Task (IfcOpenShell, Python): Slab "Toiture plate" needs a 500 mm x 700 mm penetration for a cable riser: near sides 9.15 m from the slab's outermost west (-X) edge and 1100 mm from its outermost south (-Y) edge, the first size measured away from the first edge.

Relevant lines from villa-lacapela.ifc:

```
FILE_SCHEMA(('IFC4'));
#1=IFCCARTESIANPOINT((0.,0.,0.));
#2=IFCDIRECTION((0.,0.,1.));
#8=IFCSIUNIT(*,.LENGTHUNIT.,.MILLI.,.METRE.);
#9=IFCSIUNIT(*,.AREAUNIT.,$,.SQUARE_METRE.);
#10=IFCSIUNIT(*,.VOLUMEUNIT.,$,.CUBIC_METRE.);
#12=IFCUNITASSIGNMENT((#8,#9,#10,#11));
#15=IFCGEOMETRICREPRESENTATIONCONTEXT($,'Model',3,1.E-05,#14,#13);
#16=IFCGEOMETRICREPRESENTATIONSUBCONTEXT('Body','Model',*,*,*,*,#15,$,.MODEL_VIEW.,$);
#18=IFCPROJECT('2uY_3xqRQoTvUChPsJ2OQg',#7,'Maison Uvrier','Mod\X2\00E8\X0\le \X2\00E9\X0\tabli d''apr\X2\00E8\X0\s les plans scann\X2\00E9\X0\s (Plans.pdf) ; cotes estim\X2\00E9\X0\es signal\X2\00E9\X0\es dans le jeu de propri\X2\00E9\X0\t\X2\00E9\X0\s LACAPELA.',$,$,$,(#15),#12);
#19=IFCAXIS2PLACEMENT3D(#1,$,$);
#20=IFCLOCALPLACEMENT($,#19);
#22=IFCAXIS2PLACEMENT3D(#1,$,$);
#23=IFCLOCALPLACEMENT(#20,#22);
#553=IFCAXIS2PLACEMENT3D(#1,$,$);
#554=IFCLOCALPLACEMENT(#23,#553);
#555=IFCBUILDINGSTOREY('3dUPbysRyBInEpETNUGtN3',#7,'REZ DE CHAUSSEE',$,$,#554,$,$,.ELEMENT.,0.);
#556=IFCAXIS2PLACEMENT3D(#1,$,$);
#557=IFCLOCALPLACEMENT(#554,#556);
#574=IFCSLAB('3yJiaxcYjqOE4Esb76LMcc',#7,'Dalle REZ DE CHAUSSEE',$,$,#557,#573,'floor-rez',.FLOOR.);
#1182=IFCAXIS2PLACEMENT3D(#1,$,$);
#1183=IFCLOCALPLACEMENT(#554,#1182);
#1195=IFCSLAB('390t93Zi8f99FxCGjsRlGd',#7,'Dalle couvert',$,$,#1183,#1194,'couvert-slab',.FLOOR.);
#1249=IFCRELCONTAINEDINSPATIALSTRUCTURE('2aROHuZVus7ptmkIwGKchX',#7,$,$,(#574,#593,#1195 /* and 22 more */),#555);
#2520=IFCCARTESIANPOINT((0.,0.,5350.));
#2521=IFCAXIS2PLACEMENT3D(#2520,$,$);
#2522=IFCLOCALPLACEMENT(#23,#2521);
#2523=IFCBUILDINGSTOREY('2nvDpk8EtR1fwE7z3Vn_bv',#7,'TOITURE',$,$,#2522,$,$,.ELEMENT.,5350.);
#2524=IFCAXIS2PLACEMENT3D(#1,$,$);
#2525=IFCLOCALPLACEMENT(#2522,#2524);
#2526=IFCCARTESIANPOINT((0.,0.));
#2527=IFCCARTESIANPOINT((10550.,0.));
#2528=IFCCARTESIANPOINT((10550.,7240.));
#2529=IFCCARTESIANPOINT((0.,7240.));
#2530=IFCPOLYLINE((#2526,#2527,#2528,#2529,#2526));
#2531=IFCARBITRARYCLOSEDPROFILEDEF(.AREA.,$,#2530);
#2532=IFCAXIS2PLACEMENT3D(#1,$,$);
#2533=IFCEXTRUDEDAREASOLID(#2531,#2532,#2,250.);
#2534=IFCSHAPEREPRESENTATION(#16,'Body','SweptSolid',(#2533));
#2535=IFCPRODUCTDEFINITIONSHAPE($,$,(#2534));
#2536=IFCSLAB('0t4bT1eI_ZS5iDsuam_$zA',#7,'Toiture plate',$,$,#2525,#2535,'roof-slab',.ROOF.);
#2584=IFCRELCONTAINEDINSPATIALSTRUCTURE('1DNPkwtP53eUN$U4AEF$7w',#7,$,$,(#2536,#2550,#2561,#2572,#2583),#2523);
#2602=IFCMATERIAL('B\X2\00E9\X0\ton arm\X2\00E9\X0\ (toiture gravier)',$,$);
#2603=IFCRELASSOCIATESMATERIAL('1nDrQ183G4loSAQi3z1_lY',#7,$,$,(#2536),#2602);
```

```python
import numpy as np
import ifcopenshell
import ifcopenshell.api.feature
import ifcopenshell.api.geometry
import ifcopenshell.api.root
import ifcopenshell.geom
import ifcopenshell.util.placement
import ifcopenshell.util.representation
import ifcopenshell.util.shape
import ifcopenshell.util.unit

model = ifcopenshell.open("villa-lacapela.ifc")
unit_scale = ifcopenshell.util.unit.calculate_unit_scale(model)
settings = ifcopenshell.geom.settings()


def volume(element):
    """Net volume in cubic metres, openings subtracted."""
    shape = ifcopenshell.geom.create_shape(settings, element)
    return ifcopenshell.util.shape.get_volume(shape.geometry)


slab = model.by_guid("0t4bT1eI_ZS5iDsuam_$zA")
before = volume(slab)

# Extent in the slab's own axes, in metres. The edges named are its -X and -Y sides.
slab_shape = ifcopenshell.geom.create_shape(settings, slab)
vertices = ifcopenshell.util.shape.get_vertices(slab_shape.geometry)
x_min, y_min, bottom = vertices.min(axis=0)
top = vertices[:, 2].max()

opening = ifcopenshell.api.root.create_entity(model, ifc_class="IfcOpeningElement", name="Cable riser opening", predefined_type="OPENING")
context = ifcopenshell.util.representation.get_context(model, "Model", "Body", "MODEL_VIEW")
width, depth = 0.5, 0.7
outline = [(0.0, 0.0), (width, 0.0), (width, depth), (0.0, depth), (0.0, 0.0)]
# Overshoot both faces by 50 mm so the cut is clean.
shape = ifcopenshell.api.geometry.add_slab_representation(
    model, context=context, depth=top - bottom + 0.1, polyline=outline
)
ifcopenshell.api.geometry.assign_representation(model, product=opening, representation=shape)

matrix = ifcopenshell.util.placement.get_local_placement(slab.ObjectPlacement)
matrix[:, 3] = matrix @ np.append(np.array([x_min + 9.15, y_min + 1.1, bottom - 0.05]) / unit_scale, 1.0)
ifcopenshell.api.geometry.edit_object_placement(model, product=opening, matrix=matrix, is_si=False)
ifcopenshell.api.feature.add_feature(model, feature=opening, element=slab)

after = volume(slab)

print(f"slab volume {before:.3f} -> {after:.3f} m3")

model.write("villa-lacapela-out.ifc")
```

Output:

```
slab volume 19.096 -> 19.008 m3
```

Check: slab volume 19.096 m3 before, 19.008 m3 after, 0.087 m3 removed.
